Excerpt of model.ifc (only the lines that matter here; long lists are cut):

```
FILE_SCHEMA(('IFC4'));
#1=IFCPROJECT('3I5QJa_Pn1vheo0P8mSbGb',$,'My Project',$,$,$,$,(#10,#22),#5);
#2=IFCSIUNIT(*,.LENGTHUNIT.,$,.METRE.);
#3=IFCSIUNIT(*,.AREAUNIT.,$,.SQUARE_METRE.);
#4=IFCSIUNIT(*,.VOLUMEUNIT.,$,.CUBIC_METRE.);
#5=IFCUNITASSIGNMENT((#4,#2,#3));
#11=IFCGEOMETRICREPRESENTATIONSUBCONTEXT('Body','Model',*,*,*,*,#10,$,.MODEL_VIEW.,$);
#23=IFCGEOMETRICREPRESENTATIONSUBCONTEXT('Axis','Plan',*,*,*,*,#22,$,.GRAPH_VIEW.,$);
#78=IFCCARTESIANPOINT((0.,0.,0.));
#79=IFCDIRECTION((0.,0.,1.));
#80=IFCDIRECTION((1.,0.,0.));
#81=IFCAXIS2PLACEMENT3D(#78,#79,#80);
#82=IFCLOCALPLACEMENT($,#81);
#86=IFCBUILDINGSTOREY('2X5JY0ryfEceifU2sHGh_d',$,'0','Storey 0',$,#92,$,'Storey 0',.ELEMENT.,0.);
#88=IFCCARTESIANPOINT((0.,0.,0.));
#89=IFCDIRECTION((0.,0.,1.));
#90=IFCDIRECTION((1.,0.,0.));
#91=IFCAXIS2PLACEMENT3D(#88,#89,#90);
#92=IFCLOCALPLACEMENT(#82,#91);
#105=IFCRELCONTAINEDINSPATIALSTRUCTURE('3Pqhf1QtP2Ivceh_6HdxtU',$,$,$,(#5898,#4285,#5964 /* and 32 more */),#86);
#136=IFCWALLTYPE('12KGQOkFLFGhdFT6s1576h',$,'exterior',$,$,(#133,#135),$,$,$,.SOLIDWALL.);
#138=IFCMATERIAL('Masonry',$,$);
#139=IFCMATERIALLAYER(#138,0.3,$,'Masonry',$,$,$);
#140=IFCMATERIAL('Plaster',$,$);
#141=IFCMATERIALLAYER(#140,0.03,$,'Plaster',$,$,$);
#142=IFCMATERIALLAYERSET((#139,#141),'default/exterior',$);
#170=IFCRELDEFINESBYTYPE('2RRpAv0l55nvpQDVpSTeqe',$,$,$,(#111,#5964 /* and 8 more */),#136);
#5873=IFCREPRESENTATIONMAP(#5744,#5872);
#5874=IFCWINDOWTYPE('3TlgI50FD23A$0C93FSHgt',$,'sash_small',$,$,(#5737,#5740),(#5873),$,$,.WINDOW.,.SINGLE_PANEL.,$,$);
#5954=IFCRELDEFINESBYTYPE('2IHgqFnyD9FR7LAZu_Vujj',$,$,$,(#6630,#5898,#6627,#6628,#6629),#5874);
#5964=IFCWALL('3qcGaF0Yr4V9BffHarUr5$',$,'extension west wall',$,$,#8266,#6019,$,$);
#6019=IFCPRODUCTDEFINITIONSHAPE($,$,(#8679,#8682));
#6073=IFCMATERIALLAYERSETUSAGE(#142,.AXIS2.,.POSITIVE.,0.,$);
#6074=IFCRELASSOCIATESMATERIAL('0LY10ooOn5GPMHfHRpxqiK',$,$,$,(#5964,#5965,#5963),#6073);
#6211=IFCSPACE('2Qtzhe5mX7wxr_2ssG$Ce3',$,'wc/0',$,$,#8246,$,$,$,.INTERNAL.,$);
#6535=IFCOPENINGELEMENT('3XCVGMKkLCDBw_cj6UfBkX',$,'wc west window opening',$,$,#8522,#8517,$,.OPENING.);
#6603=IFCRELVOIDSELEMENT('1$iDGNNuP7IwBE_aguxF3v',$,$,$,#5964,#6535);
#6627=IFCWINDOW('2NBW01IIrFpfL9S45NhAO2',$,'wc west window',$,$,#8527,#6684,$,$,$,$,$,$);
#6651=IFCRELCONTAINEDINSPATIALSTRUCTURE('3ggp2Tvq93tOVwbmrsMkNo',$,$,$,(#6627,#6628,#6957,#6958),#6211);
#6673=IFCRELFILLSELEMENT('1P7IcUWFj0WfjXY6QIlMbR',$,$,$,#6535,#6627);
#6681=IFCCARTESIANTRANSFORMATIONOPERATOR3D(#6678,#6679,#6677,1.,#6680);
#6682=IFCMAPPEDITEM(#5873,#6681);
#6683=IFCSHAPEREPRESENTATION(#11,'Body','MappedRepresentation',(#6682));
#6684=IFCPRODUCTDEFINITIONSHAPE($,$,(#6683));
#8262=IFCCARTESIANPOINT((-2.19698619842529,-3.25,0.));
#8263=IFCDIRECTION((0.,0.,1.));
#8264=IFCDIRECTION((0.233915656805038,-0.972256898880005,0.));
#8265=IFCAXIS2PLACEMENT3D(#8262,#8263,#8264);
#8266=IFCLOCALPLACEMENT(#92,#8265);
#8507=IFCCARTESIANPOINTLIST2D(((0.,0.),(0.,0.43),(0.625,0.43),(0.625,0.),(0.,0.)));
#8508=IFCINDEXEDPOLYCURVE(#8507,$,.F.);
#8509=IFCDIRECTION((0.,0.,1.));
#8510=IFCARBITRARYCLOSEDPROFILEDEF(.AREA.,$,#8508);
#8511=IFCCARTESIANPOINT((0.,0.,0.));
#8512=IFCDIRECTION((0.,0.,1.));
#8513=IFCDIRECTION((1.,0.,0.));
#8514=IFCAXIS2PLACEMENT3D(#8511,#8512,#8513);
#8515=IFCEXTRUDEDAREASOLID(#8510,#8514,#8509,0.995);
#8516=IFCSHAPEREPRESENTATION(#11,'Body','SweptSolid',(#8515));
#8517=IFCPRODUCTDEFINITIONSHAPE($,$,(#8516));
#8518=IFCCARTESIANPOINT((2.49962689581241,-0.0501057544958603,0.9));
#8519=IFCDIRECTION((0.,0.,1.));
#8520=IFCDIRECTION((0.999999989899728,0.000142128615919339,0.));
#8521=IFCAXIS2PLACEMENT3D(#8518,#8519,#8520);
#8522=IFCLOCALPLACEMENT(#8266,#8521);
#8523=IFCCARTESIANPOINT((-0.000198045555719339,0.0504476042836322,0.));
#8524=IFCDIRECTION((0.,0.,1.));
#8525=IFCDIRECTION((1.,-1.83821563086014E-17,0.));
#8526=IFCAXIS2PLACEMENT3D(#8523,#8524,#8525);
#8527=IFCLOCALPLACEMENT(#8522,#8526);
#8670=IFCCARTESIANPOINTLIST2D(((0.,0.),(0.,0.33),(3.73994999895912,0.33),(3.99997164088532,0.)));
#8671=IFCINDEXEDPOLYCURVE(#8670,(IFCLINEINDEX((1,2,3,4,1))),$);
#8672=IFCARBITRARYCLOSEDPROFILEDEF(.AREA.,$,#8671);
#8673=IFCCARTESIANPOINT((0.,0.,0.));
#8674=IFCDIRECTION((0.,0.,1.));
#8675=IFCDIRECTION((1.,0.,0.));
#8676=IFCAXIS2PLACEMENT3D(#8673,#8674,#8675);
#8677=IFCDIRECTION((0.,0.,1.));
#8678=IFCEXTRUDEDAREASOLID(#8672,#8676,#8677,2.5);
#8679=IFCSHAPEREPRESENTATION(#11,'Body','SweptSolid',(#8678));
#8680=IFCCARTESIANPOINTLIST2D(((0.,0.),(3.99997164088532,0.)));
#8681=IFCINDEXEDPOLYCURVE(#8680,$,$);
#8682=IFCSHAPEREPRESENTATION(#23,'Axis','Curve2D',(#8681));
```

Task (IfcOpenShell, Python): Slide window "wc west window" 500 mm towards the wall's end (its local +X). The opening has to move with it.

```python
import ifcopenshell
import ifcopenshell.api.geometry
import ifcopenshell.util.placement
import ifcopenshell.util.unit

model = ifcopenshell.open("model.ifc")
unit_scale = ifcopenshell.util.unit.calculate_unit_scale(model)

window = model.by_guid("2NBW01IIrFpfL9S45NhAO2")
opening = window.FillsVoids[0].RelatingOpeningElement
wall = opening.VoidsElements[0].RelatingBuildingElement

wall_matrix = ifcopenshell.util.placement.get_local_placement(wall.ObjectPlacement)
shift = wall_matrix[:3, 0] * 0.5 / unit_scale
before = ifcopenshell.util.placement.get_local_placement(window.ObjectPlacement)[:3, 3].copy()

# The window is placed relative to its opening, so it follows when the opening moves.
matrix = ifcopenshell.util.placement.get_local_placement(opening.ObjectPlacement)
matrix[:3, 3] += shift
ifcopenshell.api.geometry.edit_object_placement(
    model, product=opening, matrix=matrix, is_si=False, should_transform_children=True
)

after = ifcopenshell.util.placement.get_local_placement(window.ObjectPlacement)[:3, 3]
print("window moved by", (after - before).round(3) + 0.0)

model.write("model_updated.ifc")
```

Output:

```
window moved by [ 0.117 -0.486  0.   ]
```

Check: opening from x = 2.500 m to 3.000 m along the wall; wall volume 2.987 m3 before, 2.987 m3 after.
